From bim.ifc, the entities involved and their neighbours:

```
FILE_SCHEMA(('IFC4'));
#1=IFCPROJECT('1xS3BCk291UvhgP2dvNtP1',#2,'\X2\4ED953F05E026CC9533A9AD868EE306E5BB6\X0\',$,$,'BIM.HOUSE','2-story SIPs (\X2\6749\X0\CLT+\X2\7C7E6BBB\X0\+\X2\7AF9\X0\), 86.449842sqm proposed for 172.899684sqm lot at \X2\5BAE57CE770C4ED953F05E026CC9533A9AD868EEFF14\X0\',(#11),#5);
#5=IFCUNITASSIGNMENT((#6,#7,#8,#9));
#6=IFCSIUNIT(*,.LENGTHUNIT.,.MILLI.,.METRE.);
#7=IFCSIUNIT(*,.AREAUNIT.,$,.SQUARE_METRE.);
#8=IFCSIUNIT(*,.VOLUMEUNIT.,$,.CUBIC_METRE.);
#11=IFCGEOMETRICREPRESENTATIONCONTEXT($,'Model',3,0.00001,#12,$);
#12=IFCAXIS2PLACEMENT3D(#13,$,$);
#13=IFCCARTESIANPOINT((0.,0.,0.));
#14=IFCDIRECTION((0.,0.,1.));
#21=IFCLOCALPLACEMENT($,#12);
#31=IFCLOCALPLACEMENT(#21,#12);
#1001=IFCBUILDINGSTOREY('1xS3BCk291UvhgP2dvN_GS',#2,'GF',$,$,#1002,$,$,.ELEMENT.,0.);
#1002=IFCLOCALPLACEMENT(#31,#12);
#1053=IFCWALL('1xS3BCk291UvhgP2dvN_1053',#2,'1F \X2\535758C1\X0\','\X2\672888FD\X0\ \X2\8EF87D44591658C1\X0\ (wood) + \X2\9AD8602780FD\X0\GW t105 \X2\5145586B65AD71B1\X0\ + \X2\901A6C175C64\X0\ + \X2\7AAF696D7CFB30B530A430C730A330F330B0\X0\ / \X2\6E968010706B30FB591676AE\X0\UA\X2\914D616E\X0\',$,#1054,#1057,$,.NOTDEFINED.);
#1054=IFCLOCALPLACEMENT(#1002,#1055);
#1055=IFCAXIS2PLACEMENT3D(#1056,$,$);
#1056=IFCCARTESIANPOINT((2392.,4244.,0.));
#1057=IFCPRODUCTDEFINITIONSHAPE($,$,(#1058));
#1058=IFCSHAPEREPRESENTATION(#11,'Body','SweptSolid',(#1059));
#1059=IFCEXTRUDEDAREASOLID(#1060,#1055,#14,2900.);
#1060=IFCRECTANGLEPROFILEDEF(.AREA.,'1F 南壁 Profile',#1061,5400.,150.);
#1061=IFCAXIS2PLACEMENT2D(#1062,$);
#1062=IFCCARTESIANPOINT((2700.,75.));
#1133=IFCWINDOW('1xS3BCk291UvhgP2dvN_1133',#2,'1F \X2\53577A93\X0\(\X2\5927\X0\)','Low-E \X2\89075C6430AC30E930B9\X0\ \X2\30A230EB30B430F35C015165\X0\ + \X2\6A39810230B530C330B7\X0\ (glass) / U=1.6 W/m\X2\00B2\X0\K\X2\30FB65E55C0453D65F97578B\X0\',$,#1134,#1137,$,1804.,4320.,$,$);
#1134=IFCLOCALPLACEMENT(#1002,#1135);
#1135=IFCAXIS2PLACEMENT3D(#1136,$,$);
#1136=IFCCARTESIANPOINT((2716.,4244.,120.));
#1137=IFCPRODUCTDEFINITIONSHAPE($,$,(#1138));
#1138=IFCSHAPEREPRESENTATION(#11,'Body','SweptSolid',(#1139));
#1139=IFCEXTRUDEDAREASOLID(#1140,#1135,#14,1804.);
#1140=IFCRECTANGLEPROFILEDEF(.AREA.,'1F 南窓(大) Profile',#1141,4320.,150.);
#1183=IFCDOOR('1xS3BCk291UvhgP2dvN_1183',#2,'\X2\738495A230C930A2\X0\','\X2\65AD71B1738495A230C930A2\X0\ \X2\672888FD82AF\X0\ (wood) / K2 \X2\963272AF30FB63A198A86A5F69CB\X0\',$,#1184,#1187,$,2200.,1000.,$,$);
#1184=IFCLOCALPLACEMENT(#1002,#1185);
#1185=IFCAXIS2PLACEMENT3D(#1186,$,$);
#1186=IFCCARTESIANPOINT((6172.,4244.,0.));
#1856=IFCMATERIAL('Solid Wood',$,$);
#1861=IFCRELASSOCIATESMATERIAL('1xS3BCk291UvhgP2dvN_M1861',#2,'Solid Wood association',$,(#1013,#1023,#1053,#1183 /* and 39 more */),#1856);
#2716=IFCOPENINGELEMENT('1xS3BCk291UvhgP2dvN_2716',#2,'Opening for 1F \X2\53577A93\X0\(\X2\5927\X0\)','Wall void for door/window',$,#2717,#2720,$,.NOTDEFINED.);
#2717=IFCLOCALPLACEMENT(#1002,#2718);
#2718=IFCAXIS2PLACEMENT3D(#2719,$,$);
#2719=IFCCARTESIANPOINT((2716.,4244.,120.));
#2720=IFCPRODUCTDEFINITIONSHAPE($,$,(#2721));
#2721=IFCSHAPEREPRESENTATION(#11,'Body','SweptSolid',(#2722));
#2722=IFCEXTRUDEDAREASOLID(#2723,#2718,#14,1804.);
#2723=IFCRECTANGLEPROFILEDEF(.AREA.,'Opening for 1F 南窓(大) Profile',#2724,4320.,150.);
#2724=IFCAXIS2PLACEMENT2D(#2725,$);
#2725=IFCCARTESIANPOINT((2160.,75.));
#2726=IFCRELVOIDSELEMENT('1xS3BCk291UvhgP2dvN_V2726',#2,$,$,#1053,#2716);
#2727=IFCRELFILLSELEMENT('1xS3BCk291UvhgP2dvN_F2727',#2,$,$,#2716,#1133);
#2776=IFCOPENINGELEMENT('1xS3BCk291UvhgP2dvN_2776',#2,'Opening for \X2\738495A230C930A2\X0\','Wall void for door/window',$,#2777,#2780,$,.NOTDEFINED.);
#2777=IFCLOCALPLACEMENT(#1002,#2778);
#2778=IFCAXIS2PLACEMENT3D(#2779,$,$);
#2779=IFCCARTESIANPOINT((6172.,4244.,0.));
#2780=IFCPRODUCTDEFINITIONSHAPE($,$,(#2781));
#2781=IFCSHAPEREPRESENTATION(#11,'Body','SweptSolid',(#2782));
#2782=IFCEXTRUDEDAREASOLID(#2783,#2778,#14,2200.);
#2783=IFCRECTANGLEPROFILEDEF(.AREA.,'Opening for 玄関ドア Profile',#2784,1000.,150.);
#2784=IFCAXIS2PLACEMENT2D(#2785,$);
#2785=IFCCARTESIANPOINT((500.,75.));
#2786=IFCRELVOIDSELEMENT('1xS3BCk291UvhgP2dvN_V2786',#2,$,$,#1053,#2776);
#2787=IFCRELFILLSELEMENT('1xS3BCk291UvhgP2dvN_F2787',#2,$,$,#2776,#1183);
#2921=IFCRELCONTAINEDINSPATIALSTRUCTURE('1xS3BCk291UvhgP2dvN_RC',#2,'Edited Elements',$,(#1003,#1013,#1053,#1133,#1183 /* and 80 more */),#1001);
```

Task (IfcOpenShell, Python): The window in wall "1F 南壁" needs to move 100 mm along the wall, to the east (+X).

```python
import ifcopenshell
import ifcopenshell.api.geometry
import ifcopenshell.util.placement

model = ifcopenshell.open("bim.ifc")

window = model.by_id(1133)
opening = window.FillsVoids[0].RelatingOpeningElement
wall = opening.VoidsElements[0].RelatingBuildingElement

wall_matrix = ifcopenshell.util.placement.get_local_placement(wall.ObjectPlacement)
shift = wall_matrix[:3, 0] * 100.0
before = ifcopenshell.util.placement.get_local_placement(window.ObjectPlacement)[:3, 3].copy()

# The window is not placed relative to its opening, so move both.
for product in (opening, window):
    matrix = ifcopenshell.util.placement.get_local_placement(product.ObjectPlacement)
    matrix[:3, 3] += shift
    ifcopenshell.api.geometry.edit_object_placement(model, product=product, matrix=matrix, is_si=False)

after = ifcopenshell.util.placement.get_local_placement(window.ObjectPlacement)[:3, 3]
print("window moved by", (after - before).round(3) + 0.0)

model.write("bim-out.ifc")
```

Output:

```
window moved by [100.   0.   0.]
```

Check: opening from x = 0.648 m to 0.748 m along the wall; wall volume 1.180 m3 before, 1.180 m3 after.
